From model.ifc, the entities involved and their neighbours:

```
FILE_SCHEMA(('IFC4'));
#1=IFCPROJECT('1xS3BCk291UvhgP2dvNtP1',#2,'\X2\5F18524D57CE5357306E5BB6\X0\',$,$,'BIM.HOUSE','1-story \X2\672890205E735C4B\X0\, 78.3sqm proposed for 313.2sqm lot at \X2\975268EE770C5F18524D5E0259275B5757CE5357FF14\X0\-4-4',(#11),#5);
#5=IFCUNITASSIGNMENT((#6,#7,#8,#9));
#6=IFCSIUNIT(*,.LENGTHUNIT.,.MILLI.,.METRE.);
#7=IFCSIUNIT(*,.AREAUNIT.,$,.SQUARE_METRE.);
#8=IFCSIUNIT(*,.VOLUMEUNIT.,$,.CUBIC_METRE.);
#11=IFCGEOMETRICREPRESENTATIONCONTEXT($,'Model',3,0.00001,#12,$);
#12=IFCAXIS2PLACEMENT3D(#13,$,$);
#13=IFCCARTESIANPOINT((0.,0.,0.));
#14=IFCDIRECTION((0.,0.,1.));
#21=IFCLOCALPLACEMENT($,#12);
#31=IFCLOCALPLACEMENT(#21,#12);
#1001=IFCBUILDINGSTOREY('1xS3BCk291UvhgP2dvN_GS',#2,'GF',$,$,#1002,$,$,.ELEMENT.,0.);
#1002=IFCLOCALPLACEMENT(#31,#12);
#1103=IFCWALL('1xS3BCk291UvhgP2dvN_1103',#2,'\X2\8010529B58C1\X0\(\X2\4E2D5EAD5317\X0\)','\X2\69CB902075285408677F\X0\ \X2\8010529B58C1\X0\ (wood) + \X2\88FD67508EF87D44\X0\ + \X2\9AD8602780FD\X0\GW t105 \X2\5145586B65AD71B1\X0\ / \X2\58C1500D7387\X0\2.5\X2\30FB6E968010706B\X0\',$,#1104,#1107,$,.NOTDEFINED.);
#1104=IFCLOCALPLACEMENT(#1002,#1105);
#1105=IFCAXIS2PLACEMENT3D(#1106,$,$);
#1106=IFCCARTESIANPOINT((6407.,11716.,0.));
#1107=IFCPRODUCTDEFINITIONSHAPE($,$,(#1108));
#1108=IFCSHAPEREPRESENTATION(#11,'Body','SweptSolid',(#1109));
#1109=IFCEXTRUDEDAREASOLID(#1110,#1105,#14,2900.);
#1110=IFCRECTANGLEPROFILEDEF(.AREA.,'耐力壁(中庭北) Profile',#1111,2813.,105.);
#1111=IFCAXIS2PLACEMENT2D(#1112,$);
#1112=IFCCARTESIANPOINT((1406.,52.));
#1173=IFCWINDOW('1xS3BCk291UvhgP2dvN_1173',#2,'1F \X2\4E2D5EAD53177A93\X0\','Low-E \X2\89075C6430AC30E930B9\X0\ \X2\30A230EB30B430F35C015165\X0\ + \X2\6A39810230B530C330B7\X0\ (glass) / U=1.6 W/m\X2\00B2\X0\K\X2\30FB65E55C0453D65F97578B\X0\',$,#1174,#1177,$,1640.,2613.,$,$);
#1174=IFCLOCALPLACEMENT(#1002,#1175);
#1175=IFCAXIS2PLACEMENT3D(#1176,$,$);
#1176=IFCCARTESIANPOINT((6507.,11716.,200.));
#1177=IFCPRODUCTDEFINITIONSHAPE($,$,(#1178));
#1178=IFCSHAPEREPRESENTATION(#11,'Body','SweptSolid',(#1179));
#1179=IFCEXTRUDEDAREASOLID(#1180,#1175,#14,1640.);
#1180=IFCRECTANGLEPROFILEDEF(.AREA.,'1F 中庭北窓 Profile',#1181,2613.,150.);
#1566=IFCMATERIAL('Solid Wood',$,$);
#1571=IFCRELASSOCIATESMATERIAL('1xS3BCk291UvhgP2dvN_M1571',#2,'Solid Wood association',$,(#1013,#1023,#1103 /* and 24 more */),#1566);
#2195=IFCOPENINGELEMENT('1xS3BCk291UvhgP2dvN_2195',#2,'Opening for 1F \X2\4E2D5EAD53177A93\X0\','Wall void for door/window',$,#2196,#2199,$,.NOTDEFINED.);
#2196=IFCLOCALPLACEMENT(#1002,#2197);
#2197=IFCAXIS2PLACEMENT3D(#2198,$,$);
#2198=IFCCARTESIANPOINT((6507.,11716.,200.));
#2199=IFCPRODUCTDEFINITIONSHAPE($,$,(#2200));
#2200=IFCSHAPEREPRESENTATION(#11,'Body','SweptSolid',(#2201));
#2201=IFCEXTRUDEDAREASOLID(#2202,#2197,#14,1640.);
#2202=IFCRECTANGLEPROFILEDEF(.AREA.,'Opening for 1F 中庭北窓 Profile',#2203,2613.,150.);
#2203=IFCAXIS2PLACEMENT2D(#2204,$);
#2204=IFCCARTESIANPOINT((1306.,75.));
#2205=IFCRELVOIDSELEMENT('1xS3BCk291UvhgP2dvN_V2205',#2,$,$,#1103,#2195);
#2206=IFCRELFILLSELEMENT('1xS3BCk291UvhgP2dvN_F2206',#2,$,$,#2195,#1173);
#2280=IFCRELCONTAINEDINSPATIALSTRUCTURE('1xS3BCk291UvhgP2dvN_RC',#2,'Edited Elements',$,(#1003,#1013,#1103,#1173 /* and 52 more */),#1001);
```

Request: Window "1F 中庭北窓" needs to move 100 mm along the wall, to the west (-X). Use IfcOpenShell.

```python
import ifcopenshell
import ifcopenshell.api.geometry
import ifcopenshell.util.placement
import ifcopenshell.util.unit

model = ifcopenshell.open("model.ifc")
unit_scale = ifcopenshell.util.unit.calculate_unit_scale(model)

window = model.by_id(1173)
opening = window.FillsVoids[0].RelatingOpeningElement
wall = opening.VoidsElements[0].RelatingBuildingElement

wall_matrix = ifcopenshell.util.placement.get_local_placement(wall.ObjectPlacement)
shift = wall_matrix[:3, 0] * -0.1 / unit_scale
before = ifcopenshell.util.placement.get_local_placement(window.ObjectPlacement)[:3, 3].copy()

# The window is not placed relative to its opening, so move both.
for product in (opening, window):
    matrix = ifcopenshell.util.placement.get_local_placement(product.ObjectPlacement)
    matrix[:3, 3] += shift
    ifcopenshell.api.geometry.edit_object_placement(model, product=product, matrix=matrix, is_si=False)

after = ifcopenshell.util.placement.get_local_placement(window.ObjectPlacement)[:3, 3]
print("window moved by", (after - before).round(3) + 0.0)

model.write("model-out.ifc")
```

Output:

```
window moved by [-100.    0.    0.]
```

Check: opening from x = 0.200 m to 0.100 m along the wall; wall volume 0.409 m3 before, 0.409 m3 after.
